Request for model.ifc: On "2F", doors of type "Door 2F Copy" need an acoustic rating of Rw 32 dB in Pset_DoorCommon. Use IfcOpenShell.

First a look at what the model holds.

```python
import ifcopenshell
import ifcopenshell.util.element

model = ifcopenshell.open("model.ifc")
print(model.schema)
storey = next(s for s in model.by_type("IfcBuildingStorey") if s.Name == "2F")
doors = [e for e in ifcopenshell.util.element.get_decomposition(storey) if e.is_a("IfcDoor")]
seen = {}
for e in doors:
    element_type = ifcopenshell.util.element.get_type(e)
    key = (element_type.Name if element_type != e and element_type else None, ifcopenshell.util.element.get_pset(e, "Pset_DoorCommon", "AcousticRating"))
    seen[key] = seen.get(key, 0) + 1
for (name, value), count in sorted(seen.items(), key=str):
    print(count, "x", name, "|", value)
```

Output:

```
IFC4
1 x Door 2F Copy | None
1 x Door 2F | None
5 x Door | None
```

```python
import ifcopenshell
import ifcopenshell.api.pset
import ifcopenshell.util.element

model = ifcopenshell.open("model.ifc")

storey = next(s for s in model.by_type("IfcBuildingStorey") if s.Name == "2F")
doors = [e for e in ifcopenshell.util.element.get_decomposition(storey) if e.is_a("IfcDoor")]

count = 0
for e in doors:
    element_type = ifcopenshell.util.element.get_type(e)
    if element_type in (None, e) or element_type.Name != "Door 2F Copy":
        continue
    # add_pset returns the element's existing set when there is one.
    pset = ifcopenshell.api.pset.add_pset(model, product=e, name="Pset_DoorCommon")
    ifcopenshell.api.pset.edit_pset(model, pset=pset, properties={"AcousticRating": "Rw 32 dB"})
    count += 1

print(count, "doors updated")

model.write("model-out.ifc")
```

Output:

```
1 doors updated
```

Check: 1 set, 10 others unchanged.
